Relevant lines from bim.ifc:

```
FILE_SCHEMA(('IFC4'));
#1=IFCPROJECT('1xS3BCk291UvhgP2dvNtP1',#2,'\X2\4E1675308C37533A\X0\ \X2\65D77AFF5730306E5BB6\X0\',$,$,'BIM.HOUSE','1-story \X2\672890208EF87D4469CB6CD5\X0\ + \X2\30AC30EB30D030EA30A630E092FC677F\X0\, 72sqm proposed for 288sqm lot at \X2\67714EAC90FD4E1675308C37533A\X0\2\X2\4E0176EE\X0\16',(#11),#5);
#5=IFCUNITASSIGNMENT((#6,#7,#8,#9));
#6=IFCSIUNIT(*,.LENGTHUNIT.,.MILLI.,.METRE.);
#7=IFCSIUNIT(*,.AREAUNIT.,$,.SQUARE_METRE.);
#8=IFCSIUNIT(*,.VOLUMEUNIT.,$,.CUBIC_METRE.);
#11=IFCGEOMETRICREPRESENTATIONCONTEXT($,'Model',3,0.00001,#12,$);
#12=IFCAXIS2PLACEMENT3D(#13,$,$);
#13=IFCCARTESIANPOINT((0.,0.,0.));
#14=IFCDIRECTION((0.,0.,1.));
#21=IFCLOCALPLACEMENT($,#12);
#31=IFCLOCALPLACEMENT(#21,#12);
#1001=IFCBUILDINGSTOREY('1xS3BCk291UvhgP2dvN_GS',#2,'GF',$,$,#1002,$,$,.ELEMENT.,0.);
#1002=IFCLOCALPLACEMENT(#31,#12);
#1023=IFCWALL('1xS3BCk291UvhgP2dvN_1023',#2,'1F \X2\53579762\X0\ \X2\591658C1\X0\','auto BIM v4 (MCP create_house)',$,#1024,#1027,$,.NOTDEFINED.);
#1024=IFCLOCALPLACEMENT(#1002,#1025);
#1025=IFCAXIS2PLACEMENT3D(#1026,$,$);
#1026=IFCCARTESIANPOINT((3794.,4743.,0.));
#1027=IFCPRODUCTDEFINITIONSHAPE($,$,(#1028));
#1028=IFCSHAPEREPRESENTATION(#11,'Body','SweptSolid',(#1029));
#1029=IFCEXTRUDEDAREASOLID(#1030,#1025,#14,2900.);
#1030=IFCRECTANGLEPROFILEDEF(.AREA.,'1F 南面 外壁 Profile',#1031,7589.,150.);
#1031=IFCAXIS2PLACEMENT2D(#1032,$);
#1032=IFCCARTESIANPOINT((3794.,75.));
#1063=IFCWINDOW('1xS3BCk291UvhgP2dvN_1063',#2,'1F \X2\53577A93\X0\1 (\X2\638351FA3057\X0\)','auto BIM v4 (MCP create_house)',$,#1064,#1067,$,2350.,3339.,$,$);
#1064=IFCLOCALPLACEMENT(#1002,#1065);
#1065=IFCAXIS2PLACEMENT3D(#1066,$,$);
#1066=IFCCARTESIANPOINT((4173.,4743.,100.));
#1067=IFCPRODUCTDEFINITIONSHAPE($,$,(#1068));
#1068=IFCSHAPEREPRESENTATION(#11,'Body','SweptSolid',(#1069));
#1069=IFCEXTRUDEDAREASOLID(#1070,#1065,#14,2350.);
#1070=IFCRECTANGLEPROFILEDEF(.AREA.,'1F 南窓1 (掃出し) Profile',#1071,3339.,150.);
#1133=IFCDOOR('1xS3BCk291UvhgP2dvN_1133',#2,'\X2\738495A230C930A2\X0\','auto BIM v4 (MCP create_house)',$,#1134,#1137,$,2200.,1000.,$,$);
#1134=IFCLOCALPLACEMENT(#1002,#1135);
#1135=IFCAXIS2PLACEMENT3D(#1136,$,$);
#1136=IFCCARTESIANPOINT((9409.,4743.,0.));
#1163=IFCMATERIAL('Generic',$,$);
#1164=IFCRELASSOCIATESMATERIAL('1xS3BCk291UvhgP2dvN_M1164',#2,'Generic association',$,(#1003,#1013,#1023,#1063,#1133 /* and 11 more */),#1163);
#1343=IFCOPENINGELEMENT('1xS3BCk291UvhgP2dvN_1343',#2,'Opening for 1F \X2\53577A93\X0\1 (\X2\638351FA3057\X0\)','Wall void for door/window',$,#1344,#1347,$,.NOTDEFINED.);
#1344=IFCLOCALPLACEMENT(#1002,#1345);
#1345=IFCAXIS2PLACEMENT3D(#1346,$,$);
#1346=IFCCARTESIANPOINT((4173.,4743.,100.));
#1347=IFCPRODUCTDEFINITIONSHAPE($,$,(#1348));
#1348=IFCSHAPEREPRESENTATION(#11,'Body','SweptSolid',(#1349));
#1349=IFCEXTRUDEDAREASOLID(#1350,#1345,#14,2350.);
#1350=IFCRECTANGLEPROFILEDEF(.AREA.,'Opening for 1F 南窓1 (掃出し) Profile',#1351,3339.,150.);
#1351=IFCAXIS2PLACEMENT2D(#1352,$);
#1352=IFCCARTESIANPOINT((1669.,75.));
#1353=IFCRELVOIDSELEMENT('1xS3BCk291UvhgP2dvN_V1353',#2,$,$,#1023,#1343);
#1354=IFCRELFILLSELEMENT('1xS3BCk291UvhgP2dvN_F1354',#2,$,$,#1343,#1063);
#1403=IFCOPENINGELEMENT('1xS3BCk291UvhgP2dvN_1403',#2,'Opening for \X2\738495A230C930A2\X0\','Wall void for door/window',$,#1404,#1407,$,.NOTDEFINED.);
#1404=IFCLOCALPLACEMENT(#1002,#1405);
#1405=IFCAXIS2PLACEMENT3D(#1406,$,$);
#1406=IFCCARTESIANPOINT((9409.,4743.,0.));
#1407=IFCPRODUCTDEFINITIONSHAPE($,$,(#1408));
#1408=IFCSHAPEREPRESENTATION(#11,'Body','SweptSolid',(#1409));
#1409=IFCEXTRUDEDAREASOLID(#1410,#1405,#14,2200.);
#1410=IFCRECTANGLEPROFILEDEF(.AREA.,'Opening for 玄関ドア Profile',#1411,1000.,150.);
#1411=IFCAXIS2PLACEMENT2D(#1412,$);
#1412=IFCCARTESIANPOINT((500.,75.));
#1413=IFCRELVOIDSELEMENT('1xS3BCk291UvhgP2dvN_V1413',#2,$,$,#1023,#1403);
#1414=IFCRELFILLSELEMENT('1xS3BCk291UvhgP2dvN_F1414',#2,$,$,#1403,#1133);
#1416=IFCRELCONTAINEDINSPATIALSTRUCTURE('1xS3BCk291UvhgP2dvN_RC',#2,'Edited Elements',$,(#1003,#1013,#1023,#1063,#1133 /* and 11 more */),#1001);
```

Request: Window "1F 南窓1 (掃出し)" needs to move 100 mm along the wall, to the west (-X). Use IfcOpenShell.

```python
import ifcopenshell
import ifcopenshell.api.geometry
import ifcopenshell.util.placement
import ifcopenshell.util.unit

model = ifcopenshell.open("bim.ifc")
unit_scale = ifcopenshell.util.unit.calculate_unit_scale(model)

window = model.by_guid("1xS3BCk291UvhgP2dvN_1063")
opening = window.FillsVoids[0].RelatingOpeningElement
wall = opening.VoidsElements[0].RelatingBuildingElement

wall_matrix = ifcopenshell.util.placement.get_local_placement(wall.ObjectPlacement)
shift = wall_matrix[:3, 0] * -0.1 / unit_scale
before = ifcopenshell.util.placement.get_local_placement(window.ObjectPlacement)[:3, 3].copy()

# The window is not placed relative to its opening, so move both.
for product in (opening, window):
    matrix = ifcopenshell.util.placement.get_local_placement(product.ObjectPlacement)
    matrix[:3, 3] += shift
    ifcopenshell.api.geometry.edit_object_placement(model, product=product, matrix=matrix, is_si=False)

after = ifcopenshell.util.placement.get_local_placement(window.ObjectPlacement)[:3, 3]
print("window moved by", (after - before).round(3) + 0.0)

model.write("bim_edited.ifc")
```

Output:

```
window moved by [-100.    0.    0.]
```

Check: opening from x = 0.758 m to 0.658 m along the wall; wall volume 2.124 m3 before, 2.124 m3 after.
